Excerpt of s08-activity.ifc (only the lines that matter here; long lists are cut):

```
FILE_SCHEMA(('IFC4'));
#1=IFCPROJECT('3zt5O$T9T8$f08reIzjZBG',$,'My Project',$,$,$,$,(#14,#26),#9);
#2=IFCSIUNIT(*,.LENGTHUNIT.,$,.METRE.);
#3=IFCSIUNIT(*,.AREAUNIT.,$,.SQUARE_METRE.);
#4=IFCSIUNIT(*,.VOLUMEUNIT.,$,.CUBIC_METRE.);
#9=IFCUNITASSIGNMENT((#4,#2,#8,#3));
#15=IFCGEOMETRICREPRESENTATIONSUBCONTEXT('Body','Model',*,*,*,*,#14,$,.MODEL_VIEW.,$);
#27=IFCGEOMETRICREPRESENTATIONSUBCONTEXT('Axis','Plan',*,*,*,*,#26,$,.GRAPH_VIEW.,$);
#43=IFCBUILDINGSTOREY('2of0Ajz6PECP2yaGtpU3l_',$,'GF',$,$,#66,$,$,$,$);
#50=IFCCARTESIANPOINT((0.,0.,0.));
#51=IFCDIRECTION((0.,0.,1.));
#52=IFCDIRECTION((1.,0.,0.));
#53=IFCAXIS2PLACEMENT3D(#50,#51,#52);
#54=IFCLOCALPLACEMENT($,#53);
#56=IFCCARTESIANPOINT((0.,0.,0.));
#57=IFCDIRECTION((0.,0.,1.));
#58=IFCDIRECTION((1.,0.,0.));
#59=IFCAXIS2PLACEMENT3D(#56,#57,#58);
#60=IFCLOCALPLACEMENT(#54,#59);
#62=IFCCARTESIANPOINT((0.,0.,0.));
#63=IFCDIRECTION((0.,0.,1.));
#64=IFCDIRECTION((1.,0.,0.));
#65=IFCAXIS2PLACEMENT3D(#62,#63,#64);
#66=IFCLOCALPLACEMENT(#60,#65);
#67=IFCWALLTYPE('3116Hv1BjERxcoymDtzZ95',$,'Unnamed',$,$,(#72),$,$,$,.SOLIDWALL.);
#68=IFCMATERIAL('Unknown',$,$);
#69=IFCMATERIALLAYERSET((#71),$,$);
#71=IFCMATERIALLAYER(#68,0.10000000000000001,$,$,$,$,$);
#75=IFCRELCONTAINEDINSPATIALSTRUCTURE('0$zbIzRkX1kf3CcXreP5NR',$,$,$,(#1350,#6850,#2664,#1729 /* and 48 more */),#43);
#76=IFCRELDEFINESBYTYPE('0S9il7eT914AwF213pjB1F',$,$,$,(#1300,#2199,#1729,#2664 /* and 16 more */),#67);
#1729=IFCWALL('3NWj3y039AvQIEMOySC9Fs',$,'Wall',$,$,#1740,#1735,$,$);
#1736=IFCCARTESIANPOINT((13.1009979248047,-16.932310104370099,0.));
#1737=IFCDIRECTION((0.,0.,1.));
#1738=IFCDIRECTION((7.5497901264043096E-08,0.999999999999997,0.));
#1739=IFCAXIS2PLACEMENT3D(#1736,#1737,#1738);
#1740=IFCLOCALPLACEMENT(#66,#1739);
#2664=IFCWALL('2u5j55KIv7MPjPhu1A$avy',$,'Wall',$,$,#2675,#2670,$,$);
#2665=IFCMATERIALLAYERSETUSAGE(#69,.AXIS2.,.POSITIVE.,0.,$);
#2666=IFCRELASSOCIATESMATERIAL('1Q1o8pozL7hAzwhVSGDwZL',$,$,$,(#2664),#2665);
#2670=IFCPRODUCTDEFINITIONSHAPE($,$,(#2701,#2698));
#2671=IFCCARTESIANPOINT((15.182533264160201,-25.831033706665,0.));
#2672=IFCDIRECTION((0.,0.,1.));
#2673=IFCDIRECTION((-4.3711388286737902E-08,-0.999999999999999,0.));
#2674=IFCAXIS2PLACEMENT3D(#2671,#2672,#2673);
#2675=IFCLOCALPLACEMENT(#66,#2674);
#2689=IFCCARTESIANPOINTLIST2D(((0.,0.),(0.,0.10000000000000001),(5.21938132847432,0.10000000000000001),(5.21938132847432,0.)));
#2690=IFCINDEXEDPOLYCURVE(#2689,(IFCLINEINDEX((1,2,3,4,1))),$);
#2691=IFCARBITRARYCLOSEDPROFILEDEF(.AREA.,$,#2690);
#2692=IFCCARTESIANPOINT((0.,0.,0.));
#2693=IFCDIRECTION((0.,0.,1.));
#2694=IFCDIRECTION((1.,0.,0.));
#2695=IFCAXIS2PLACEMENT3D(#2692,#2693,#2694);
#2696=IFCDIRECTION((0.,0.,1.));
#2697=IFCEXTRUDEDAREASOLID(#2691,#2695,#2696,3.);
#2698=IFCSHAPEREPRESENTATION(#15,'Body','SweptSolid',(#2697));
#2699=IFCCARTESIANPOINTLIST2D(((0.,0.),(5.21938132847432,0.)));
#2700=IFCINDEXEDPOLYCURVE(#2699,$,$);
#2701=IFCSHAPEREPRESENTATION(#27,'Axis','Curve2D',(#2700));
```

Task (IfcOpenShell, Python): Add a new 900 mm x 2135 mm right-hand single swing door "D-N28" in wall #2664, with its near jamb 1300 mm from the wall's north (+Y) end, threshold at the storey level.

```python
import numpy as np
import ifcopenshell
import ifcopenshell.api.feature
import ifcopenshell.api.geometry
import ifcopenshell.api.root
import ifcopenshell.api.spatial
import ifcopenshell.geom
import ifcopenshell.util.element
import ifcopenshell.util.placement
import ifcopenshell.util.representation
import ifcopenshell.util.shape
import ifcopenshell.util.unit

model = ifcopenshell.open("s08-activity.ifc")
unit_scale = ifcopenshell.util.unit.calculate_unit_scale(model)
settings = ifcopenshell.geom.settings()


def volume(element):
    """Net volume in cubic metres, openings subtracted."""
    shape = ifcopenshell.geom.create_shape(settings, element)
    return ifcopenshell.util.shape.get_volume(shape.geometry)


wall = model.by_guid("2u5j55KIv7MPjPhu1A$avy")
storey = ifcopenshell.util.element.get_container(wall, ifc_class="IfcBuildingStorey")
context = ifcopenshell.util.representation.get_context(model, "Model", "Body", "MODEL_VIEW")
before = volume(wall)

width, height, from_end, sill = 0.9, 2.135, 1.3, 0.0  # metres

# The wall runs along its own X axis, and the end named is its -X end.
wall_shape = ifcopenshell.geom.create_shape(settings, wall)
x, y, z = ifcopenshell.util.shape.get_vertices(wall_shape.geometry).T
start = x.min() + from_end
face, thickness = float(y.min()), float(y.max() - y.min())
wall_matrix = ifcopenshell.util.placement.get_local_placement(wall.ObjectPlacement)
level = ifcopenshell.util.placement.get_local_placement(storey.ObjectPlacement)[2, 3]


def in_wall(x, y):
    """Placement at x, y metres in the wall's axes, at sill height."""
    matrix = wall_matrix.copy()
    matrix[:, 3] = wall_matrix @ np.array([x / unit_scale, y / unit_scale, 0.0, 1.0])
    matrix[2, 3] = level + sill / unit_scale
    return matrix


# Opening: a box that overshoots both wall faces by 50 mm.
opening = ifcopenshell.api.root.create_entity(model, ifc_class="IfcOpeningElement", predefined_type="OPENING")
box = ifcopenshell.api.geometry.add_wall_representation(
    model, context=context, length=width, height=height, thickness=thickness + 0.1
)
ifcopenshell.api.geometry.assign_representation(model, product=opening, representation=box)
ifcopenshell.api.geometry.edit_object_placement(model, product=opening, matrix=in_wall(start, face - 0.05), is_si=False)
ifcopenshell.api.feature.add_feature(model, feature=opening, element=wall)

door = ifcopenshell.api.root.create_entity(model, ifc_class="IfcDoor", name="D-N28", predefined_type="DOOR")
door.OverallWidth, door.OverallHeight = width / unit_scale, height / unit_scale
door.OperationType = "SINGLE_SWING_RIGHT"
body = ifcopenshell.api.geometry.add_door_representation(
    model,
    context=context,
    overall_width=door.OverallWidth,
    overall_height=door.OverallHeight,
    operation_type="SINGLE_SWING_RIGHT",
    lining_properties={"LiningDepth": thickness / unit_scale, "ThresholdDepth": thickness / unit_scale},
)
ifcopenshell.api.geometry.assign_representation(model, product=door, representation=body)
ifcopenshell.api.spatial.assign_container(model, products=[door], relating_structure=storey)
ifcopenshell.api.feature.add_filling(model, opening=opening, element=door)

# The lining spans the wall, so the door starts at the wall face.
ifcopenshell.api.geometry.edit_object_placement(model, product=door, matrix=in_wall(start, face), is_si=False)

after = volume(wall)

print(f"wall volume {before:.3f} -> {after:.3f} m3")

model.write("s08-activity_rev.ifc")
```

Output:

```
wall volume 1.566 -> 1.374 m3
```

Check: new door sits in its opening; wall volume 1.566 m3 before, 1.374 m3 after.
